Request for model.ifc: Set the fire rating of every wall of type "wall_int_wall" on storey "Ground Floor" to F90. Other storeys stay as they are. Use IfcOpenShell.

First a look at what the model holds.

```python
import ifcopenshell
import ifcopenshell.util.element

model = ifcopenshell.open("model.ifc")
print(model.schema)
storey = next(s for s in model.by_type("IfcBuildingStorey") if s.Name == "Ground Floor")
walls = [e for e in ifcopenshell.util.element.get_decomposition(storey) if e.is_a("IfcWall")]
seen = {}
for e in walls:
    element_type = ifcopenshell.util.element.get_type(e)
    key = (element_type.Name if element_type != e and element_type else None, ifcopenshell.util.element.get_pset(e, "Pset_WallCommon", "FireRating"))
    seen[key] = seen.get(key, 0) + 1
for (name, value), count in sorted(seen.items(), key=str):
    print(count, "x", name, "|", value)
```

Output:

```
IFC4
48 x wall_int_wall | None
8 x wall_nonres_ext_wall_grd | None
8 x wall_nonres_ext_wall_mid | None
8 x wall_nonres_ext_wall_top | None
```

```python
import ifcopenshell
import ifcopenshell.api.pset
import ifcopenshell.util.element

model = ifcopenshell.open("model.ifc")

storey = next(s for s in model.by_type("IfcBuildingStorey") if s.Name == "Ground Floor")
walls = [e for e in ifcopenshell.util.element.get_decomposition(storey) if e.is_a("IfcWall")]

count = 0
for e in walls:
    element_type = ifcopenshell.util.element.get_type(e)
    if element_type in (None, e) or element_type.Name != "wall_int_wall":
        continue
    # add_pset returns the element's existing set when there is one.
    pset = ifcopenshell.api.pset.add_pset(model, product=e, name="Pset_WallCommon")
    ifcopenshell.api.pset.edit_pset(model, pset=pset, properties={"FireRating": "F90"})
    count += 1

print(count, "walls updated")

model.write("model-out.ifc")
```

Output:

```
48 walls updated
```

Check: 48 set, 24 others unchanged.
